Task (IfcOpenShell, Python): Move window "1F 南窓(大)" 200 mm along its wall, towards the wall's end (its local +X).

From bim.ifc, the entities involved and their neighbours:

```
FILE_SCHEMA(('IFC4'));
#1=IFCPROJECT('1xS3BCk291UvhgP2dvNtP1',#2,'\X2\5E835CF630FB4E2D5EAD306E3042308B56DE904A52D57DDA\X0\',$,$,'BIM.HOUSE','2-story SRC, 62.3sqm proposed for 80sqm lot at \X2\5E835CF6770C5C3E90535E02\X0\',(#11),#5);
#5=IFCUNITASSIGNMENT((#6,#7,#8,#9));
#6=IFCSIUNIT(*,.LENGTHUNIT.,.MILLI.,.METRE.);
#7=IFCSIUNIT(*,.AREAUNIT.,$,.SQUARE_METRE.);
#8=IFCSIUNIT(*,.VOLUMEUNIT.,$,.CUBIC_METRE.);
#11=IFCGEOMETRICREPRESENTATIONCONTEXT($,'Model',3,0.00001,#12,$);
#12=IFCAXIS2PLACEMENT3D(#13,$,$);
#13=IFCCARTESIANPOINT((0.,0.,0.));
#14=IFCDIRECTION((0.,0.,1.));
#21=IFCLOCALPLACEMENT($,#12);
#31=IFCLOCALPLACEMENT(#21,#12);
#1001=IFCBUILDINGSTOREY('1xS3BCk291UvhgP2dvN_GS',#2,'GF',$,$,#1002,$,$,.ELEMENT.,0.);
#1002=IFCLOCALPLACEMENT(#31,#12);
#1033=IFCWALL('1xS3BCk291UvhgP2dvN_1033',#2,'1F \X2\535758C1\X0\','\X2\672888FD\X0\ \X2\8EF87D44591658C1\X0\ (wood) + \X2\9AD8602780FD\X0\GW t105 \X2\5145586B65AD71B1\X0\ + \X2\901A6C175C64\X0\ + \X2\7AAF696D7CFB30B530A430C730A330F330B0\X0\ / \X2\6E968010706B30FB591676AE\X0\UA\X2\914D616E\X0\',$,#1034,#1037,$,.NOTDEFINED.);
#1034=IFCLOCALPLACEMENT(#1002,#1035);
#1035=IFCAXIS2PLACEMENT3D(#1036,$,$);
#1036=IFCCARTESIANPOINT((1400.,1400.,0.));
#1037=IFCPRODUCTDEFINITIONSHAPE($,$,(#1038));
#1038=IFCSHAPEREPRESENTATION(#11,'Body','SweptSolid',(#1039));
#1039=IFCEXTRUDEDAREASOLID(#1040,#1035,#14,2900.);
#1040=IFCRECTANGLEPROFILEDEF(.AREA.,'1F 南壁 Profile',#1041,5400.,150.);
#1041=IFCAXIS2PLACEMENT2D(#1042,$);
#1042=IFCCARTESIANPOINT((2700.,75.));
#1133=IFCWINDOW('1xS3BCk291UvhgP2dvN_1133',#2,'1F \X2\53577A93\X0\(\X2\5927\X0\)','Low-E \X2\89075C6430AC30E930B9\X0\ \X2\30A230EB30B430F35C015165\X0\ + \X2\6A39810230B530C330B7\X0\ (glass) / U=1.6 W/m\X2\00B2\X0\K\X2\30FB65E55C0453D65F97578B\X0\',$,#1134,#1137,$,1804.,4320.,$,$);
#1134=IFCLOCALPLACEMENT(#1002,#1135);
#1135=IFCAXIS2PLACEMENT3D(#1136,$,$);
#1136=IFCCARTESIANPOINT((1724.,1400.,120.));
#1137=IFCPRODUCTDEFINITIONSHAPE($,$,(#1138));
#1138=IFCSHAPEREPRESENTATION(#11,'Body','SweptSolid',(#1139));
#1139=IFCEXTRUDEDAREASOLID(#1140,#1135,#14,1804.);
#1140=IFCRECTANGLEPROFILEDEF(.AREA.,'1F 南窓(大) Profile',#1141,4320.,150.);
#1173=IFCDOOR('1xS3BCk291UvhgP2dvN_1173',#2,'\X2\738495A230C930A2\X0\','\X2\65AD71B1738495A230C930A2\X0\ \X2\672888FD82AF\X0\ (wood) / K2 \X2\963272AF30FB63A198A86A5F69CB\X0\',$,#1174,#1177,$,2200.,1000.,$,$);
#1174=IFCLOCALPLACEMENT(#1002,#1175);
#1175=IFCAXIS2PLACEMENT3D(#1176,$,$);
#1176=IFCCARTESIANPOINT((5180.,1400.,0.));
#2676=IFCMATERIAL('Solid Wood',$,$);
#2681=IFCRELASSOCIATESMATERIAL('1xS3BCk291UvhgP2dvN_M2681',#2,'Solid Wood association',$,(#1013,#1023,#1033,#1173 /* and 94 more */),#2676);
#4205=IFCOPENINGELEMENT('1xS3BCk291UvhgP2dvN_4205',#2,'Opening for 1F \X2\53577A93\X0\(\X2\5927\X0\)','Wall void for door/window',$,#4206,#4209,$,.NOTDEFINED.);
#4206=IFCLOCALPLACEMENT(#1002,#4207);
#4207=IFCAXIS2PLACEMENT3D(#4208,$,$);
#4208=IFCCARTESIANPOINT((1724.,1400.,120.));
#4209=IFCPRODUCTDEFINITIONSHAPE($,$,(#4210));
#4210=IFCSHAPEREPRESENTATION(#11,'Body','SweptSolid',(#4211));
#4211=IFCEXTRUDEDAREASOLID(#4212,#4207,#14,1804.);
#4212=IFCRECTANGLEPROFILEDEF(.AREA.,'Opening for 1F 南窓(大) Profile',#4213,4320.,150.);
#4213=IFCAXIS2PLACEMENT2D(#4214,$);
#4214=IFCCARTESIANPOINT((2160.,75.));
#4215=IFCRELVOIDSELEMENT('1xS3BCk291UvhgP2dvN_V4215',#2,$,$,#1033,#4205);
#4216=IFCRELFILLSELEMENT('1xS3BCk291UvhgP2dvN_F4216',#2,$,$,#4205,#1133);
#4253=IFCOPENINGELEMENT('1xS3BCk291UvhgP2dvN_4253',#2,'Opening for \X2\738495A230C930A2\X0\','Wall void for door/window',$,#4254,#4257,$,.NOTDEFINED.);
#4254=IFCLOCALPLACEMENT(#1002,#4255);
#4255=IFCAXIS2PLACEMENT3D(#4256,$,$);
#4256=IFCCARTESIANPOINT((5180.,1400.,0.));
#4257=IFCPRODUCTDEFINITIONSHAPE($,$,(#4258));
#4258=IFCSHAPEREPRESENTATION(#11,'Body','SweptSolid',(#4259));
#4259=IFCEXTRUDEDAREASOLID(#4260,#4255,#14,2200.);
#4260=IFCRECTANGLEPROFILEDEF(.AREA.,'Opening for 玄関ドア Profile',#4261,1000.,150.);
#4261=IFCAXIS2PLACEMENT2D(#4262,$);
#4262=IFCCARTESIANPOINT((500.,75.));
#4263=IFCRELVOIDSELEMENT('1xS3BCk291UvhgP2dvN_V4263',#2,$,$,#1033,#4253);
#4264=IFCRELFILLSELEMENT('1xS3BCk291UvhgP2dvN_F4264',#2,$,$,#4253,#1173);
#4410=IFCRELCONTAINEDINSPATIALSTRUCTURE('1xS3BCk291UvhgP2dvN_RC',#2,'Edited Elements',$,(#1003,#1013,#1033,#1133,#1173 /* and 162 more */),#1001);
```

```python
import ifcopenshell
import ifcopenshell.api.geometry
import ifcopenshell.util.placement

model = ifcopenshell.open("bim.ifc")

window = model.by_id(1133)
opening = window.FillsVoids[0].RelatingOpeningElement
wall = opening.VoidsElements[0].RelatingBuildingElement

wall_matrix = ifcopenshell.util.placement.get_local_placement(wall.ObjectPlacement)
shift = wall_matrix[:3, 0] * 200.0
before = ifcopenshell.util.placement.get_local_placement(window.ObjectPlacement)[:3, 3].copy()

# The window is not placed relative to its opening, so move both.
for product in (opening, window):
    matrix = ifcopenshell.util.placement.get_local_placement(product.ObjectPlacement)
    matrix[:3, 3] += shift
    ifcopenshell.api.geometry.edit_object_placement(model, product=product, matrix=matrix, is_si=False)

after = ifcopenshell.util.placement.get_local_placement(window.ObjectPlacement)[:3, 3]
print("window moved by", (after - before).round(3) + 0.0)

model.write("bim_rev.ifc")
```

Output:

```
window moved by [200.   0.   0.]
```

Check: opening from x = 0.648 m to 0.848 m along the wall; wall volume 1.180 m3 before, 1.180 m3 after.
